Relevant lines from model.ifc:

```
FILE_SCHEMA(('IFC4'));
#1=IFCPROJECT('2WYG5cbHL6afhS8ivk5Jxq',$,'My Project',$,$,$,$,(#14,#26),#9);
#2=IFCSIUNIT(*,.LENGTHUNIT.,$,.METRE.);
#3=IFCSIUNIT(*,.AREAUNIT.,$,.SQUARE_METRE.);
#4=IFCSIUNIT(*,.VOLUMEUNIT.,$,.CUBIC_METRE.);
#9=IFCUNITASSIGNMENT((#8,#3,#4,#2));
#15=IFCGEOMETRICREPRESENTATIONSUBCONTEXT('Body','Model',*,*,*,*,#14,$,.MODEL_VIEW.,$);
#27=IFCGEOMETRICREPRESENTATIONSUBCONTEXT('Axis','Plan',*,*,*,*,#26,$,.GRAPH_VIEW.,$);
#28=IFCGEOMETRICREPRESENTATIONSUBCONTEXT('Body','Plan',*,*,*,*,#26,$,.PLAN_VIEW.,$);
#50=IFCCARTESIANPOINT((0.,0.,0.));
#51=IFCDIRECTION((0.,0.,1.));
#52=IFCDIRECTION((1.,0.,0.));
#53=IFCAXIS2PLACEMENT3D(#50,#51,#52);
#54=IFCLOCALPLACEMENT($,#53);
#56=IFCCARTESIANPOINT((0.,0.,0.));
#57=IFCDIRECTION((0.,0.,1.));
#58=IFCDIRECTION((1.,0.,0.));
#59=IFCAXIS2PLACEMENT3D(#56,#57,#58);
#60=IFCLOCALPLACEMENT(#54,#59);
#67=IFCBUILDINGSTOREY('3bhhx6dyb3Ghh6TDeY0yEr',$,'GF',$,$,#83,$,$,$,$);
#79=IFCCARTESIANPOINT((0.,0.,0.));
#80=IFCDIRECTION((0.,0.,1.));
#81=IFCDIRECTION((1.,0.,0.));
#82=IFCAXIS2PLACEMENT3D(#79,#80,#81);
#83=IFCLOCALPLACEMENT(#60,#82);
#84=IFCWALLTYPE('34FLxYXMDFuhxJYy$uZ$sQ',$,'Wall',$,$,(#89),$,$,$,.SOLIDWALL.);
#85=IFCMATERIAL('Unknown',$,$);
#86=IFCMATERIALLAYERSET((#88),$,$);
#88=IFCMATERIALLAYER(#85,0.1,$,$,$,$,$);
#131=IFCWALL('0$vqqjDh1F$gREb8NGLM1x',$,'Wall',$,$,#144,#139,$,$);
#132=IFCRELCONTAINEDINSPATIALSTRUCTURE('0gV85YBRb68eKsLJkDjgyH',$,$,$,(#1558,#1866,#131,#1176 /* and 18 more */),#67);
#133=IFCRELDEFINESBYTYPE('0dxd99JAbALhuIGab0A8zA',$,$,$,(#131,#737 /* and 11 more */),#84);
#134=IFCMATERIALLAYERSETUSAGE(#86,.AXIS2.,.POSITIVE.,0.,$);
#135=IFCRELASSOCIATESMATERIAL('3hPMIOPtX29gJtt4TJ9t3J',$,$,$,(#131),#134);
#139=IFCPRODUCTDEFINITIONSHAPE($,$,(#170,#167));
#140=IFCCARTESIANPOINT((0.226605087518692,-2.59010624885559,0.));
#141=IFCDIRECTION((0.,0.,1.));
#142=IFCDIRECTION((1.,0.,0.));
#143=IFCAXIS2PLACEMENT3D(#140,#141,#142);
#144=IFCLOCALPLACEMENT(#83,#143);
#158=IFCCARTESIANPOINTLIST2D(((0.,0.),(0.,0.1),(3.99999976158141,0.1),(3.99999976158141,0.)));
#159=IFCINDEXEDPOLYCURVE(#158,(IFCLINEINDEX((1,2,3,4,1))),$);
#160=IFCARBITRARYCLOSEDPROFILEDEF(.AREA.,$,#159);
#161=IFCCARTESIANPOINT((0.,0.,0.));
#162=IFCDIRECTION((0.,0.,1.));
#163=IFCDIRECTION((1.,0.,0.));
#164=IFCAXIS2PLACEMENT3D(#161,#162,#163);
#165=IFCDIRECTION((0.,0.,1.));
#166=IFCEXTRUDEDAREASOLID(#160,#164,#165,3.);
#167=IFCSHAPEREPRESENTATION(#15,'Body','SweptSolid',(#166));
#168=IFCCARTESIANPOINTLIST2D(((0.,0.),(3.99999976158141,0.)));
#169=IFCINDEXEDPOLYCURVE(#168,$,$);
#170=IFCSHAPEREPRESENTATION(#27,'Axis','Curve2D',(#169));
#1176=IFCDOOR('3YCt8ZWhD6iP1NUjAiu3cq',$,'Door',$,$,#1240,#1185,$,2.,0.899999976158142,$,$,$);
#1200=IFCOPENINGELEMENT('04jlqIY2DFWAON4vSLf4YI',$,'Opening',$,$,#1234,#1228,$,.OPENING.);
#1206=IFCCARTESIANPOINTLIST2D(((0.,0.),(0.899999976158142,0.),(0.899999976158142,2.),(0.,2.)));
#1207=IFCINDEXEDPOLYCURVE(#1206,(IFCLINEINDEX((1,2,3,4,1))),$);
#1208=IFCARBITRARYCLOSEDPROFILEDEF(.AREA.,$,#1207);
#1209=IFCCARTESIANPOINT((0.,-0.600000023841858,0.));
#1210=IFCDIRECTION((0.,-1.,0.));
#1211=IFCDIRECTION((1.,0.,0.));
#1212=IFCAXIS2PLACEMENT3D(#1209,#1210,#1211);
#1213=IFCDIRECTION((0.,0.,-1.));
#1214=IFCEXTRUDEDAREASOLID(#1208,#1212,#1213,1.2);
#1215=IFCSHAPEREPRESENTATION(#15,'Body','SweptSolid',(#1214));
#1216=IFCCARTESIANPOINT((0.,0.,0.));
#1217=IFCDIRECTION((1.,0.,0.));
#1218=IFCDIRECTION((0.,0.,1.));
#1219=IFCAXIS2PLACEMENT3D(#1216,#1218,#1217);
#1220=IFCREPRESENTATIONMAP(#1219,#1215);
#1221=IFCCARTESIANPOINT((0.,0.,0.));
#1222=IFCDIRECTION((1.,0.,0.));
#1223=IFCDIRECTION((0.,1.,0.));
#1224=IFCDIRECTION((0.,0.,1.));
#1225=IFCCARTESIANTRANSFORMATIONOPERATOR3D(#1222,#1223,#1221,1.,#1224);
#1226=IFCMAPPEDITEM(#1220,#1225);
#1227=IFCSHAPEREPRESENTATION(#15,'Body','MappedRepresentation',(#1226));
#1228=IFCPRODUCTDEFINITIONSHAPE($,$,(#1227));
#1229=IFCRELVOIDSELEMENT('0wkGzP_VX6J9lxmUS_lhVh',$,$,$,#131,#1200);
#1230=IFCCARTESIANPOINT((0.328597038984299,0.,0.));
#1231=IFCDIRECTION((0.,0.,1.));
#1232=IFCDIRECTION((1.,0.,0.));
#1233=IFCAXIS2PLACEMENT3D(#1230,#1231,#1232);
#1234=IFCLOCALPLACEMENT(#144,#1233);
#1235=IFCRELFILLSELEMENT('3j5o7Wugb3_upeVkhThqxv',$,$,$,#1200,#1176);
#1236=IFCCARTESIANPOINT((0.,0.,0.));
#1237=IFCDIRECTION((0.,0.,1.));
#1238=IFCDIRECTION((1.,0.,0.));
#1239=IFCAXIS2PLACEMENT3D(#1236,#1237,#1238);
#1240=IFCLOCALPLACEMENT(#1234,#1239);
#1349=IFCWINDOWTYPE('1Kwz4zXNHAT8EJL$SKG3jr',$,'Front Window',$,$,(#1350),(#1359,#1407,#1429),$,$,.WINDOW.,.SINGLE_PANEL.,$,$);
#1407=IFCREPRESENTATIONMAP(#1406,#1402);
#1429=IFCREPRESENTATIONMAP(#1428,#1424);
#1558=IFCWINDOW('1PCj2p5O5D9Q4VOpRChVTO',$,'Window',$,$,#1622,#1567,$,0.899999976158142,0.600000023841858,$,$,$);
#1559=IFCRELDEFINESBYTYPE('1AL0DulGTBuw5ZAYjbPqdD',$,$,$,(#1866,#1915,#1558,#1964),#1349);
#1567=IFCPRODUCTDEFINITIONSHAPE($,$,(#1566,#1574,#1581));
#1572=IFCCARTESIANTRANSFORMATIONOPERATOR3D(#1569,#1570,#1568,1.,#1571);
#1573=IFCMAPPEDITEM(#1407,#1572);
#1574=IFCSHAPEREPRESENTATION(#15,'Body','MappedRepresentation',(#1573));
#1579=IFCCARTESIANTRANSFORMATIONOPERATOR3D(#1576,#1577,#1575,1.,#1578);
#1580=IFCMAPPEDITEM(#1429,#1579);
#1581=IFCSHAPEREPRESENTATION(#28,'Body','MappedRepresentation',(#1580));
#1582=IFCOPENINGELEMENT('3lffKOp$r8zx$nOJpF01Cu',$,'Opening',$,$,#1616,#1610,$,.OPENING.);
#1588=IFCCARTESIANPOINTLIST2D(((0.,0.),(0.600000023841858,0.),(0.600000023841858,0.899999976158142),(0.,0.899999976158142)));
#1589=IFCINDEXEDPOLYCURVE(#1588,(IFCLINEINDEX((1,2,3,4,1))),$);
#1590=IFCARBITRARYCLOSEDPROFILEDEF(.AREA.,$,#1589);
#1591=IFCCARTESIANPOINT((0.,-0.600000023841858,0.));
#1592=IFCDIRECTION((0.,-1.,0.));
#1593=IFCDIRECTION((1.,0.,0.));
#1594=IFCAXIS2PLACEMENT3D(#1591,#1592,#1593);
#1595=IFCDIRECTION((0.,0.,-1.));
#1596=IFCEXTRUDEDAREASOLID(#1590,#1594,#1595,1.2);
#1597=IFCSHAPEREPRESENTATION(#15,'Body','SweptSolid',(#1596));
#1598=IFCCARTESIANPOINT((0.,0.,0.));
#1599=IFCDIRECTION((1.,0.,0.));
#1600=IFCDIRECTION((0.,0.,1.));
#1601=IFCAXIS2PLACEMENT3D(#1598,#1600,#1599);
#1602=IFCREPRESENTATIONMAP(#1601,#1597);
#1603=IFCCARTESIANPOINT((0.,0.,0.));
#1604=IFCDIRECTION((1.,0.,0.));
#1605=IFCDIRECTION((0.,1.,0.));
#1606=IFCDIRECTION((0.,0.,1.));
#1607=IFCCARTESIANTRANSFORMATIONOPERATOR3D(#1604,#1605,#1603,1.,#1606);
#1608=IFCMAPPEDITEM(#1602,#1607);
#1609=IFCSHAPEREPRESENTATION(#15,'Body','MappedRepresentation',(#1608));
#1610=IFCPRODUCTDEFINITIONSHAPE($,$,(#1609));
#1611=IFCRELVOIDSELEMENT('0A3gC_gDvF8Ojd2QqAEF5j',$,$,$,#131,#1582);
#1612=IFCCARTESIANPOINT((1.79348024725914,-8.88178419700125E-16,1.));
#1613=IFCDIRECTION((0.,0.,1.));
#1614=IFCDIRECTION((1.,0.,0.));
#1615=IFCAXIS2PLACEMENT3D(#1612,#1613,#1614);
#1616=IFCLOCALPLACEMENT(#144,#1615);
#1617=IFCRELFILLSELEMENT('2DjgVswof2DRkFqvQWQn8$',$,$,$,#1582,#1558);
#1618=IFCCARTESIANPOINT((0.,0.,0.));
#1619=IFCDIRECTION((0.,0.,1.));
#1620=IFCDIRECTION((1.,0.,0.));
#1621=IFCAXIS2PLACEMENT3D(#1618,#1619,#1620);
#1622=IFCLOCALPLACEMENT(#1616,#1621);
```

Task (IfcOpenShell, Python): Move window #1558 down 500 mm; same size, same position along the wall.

```python
import numpy as np
import ifcopenshell
import ifcopenshell.api.geometry
import ifcopenshell.util.placement
import ifcopenshell.util.unit

model = ifcopenshell.open("model.ifc")
unit_scale = ifcopenshell.util.unit.calculate_unit_scale(model)

window = model.by_guid("1PCj2p5O5D9Q4VOpRChVTO")
opening = window.FillsVoids[0].RelatingOpeningElement
dz = -0.5 / unit_scale

shift = np.array([0.0, 0.0, dz])
# The window is placed relative to its opening, so it follows when the opening moves.
matrix = ifcopenshell.util.placement.get_local_placement(opening.ObjectPlacement)
matrix[:3, 3] += shift
ifcopenshell.api.geometry.edit_object_placement(
    model, product=opening, matrix=matrix, is_si=False, should_transform_children=True
)

print(f"moved by {dz * unit_scale:+.3f} m")

model.write("model_rev.ifc")
```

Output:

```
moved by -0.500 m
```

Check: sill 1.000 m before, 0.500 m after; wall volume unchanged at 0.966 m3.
